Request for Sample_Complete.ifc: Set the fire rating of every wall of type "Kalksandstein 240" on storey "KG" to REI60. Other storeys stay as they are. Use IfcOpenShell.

First a look at what the model holds.

```python
import ifcopenshell
import ifcopenshell.util.element

model = ifcopenshell.open("Sample_Complete.ifc")
print(model.schema)
storey = next(s for s in model.by_type("IfcBuildingStorey") if s.Name == "KG")
walls = [e for e in ifcopenshell.util.element.get_decomposition(storey) if e.is_a("IfcWall")]
seen = {}
for e in walls:
    element_type = ifcopenshell.util.element.get_type(e)
    key = (element_type.Name if element_type != e and element_type else None, ifcopenshell.util.element.get_pset(e, "Pset_WallCommon", "FireRating"))
    seen[key] = seen.get(key, 0) + 1
for (name, value), count in sorted(seen.items(), key=str):
    print(count, "x", name, "|", value)
```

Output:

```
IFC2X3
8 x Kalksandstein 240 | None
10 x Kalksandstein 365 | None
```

```python
import ifcopenshell
import ifcopenshell.api.pset
import ifcopenshell.util.element

model = ifcopenshell.open("Sample_Complete.ifc")

storey = next(s for s in model.by_type("IfcBuildingStorey") if s.Name == "KG")
walls = [e for e in ifcopenshell.util.element.get_decomposition(storey) if e.is_a("IfcWall")]

count = 0
for e in walls:
    element_type = ifcopenshell.util.element.get_type(e)
    if element_type in (None, e) or element_type.Name != "Kalksandstein 240":
        continue
    # add_pset returns the element's existing set when there is one.
    pset = ifcopenshell.api.pset.add_pset(model, product=e, name="Pset_WallCommon")
    ifcopenshell.api.pset.edit_pset(model, pset=pset, properties={"FireRating": "REI60"})
    count += 1

print(count, "walls updated")

model.write("Sample_Complete-out.ifc")
```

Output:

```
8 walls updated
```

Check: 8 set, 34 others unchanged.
